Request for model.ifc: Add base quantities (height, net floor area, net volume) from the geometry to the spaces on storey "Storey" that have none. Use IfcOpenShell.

First a look at what the model holds.

```python
import ifcopenshell
import ifcopenshell.util.element
import ifcopenshell.util.unit

model = ifcopenshell.open("model.ifc")
print(model.schema)
for unit_type in ("LENGTHUNIT", "AREAUNIT", "VOLUMEUNIT"):
    print(unit_type, ifcopenshell.util.unit.calculate_unit_scale(model, unit_type))
storey = next(s for s in model.by_type("IfcBuildingStorey") if s.Name == "Storey")
spaces = [e for e in ifcopenshell.util.element.get_decomposition(storey) if e.is_a("IfcSpace")]
for e in sorted(spaces, key=lambda e: e.id()):
    print(e.id(), e.is_a(), e.Name, list(ifcopenshell.util.element.get_psets(e, qtos_only=True)), sep=" | ")
```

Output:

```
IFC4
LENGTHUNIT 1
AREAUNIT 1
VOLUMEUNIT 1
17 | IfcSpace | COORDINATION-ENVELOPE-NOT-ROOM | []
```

```python
import ifcopenshell
import ifcopenshell.api.pset
import ifcopenshell.geom
import ifcopenshell.util.element
import ifcopenshell.util.shape
import ifcopenshell.util.unit

model = ifcopenshell.open("model.ifc")
unit_scale = ifcopenshell.util.unit.calculate_unit_scale(model)
area_scale = ifcopenshell.util.unit.calculate_unit_scale(model, "AREAUNIT")
volume_scale = ifcopenshell.util.unit.calculate_unit_scale(model, "VOLUMEUNIT")
settings = ifcopenshell.geom.settings()

storey = next(s for s in model.by_type("IfcBuildingStorey") if s.Name == "Storey")
spaces = [e for e in ifcopenshell.util.element.get_decomposition(storey) if e.is_a("IfcSpace")]

for e in sorted(spaces, key=lambda e: e.id()):
    if ifcopenshell.util.element.get_psets(e, qtos_only=True, should_inherit=False):
        continue
    # Geometry comes back in metres, in the element's own axes.
    shape = ifcopenshell.geom.create_shape(settings, e)
    values = {
        "Height": ifcopenshell.util.shape.get_z(shape.geometry) / unit_scale,
        "NetFloorArea": ifcopenshell.util.shape.get_footprint_area(shape.geometry) / area_scale,
        "NetVolume": ifcopenshell.util.shape.get_volume(shape.geometry) / volume_scale,
    }
    qto = ifcopenshell.api.pset.add_qto(model, product=e, name="Qto_SpaceBaseQuantities")
    ifcopenshell.api.pset.edit_qto(model, qto=qto, properties=values)
    print(e.id(), {k: round(v, 3) for k, v in values.items()})

model.write("model_rev.ifc")
```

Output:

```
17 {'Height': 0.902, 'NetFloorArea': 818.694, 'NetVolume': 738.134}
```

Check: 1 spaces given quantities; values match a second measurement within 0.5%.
